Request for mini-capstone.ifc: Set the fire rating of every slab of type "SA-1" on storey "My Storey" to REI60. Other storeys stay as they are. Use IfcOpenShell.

First a look at what the model holds.

```python
import ifcopenshell
import ifcopenshell.util.element

model = ifcopenshell.open("mini-capstone.ifc")
print(model.schema)
storey = next(s for s in model.by_type("IfcBuildingStorey") if s.Name == "My Storey")
slabs = [e for e in ifcopenshell.util.element.get_decomposition(storey) if e.is_a("IfcSlab")]
seen = {}
for e in slabs:
    element_type = ifcopenshell.util.element.get_type(e)
    key = (element_type.Name if element_type != e and element_type else None, ifcopenshell.util.element.get_pset(e, "Pset_SlabCommon", "FireRating"))
    seen[key] = seen.get(key, 0) + 1
for (name, value), count in sorted(seen.items(), key=str):
    print(count, "x", name, "|", value)
```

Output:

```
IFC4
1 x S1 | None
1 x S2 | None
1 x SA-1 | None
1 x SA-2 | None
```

```python
import ifcopenshell
import ifcopenshell.api.pset
import ifcopenshell.util.element

model = ifcopenshell.open("mini-capstone.ifc")

storey = next(s for s in model.by_type("IfcBuildingStorey") if s.Name == "My Storey")
slabs = [e for e in ifcopenshell.util.element.get_decomposition(storey) if e.is_a("IfcSlab")]

count = 0
for e in slabs:
    element_type = ifcopenshell.util.element.get_type(e)
    if element_type in (None, e) or element_type.Name != "SA-1":
        continue
    # add_pset returns the element's existing set when there is one.
    pset = ifcopenshell.api.pset.add_pset(model, product=e, name="Pset_SlabCommon")
    ifcopenshell.api.pset.edit_pset(model, pset=pset, properties={"FireRating": "REI60"})
    count += 1

print(count, "slabs updated")

model.write("mini-capstone_updated.ifc")
```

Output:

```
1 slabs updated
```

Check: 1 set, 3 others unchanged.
